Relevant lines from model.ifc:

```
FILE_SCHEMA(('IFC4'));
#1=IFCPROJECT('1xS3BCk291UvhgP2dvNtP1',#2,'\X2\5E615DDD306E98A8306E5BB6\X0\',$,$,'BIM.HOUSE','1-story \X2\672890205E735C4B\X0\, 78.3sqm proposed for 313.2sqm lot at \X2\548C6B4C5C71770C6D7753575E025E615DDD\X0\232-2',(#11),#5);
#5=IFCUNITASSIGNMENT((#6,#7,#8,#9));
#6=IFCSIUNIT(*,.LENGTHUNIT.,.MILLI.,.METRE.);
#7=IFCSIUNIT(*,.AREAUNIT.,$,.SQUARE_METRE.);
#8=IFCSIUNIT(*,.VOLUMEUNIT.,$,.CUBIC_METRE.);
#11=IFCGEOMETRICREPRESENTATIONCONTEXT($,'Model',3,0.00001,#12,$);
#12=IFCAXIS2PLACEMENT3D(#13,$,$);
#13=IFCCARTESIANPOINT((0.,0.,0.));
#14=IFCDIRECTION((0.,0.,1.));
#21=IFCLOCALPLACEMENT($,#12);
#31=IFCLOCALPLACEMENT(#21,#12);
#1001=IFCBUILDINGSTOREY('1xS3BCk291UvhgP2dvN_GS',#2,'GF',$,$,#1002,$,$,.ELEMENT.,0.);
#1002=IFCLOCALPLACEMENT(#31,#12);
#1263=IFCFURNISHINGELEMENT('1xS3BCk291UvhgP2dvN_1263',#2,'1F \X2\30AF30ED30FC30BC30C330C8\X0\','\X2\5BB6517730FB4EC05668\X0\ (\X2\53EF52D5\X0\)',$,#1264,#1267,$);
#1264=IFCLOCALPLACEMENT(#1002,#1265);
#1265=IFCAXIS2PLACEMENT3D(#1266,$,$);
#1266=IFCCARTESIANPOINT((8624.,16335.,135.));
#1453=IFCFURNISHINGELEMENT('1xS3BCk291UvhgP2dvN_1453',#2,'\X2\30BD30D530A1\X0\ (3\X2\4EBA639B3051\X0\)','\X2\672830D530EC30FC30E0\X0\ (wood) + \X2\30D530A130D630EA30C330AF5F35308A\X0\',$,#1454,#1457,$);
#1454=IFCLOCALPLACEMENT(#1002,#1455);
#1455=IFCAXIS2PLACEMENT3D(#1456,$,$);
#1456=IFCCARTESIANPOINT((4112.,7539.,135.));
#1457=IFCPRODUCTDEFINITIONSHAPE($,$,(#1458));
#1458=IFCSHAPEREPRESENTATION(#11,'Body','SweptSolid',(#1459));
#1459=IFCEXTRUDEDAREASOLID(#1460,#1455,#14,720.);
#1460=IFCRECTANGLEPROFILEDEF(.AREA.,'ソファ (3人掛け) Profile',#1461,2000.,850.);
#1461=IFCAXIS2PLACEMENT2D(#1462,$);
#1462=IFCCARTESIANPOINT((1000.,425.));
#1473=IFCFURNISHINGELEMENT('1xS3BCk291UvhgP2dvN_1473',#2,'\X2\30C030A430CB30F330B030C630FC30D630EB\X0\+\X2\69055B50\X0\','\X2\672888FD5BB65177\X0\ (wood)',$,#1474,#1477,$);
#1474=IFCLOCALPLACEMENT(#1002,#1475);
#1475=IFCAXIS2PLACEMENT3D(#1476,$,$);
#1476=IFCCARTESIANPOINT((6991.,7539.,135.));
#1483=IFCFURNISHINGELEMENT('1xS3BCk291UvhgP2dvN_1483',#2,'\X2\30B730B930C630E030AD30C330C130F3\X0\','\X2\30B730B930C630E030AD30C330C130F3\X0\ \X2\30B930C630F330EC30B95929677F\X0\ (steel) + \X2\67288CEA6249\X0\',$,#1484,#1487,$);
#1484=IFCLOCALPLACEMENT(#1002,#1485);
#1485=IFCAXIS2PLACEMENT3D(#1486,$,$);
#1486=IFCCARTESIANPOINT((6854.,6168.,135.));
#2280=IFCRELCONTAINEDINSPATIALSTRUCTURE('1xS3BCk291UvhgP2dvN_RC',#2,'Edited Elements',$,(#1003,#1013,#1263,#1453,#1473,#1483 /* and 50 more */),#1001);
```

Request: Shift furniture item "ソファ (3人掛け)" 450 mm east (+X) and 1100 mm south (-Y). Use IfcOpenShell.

```python
import ifcopenshell
import ifcopenshell.api.geometry
import ifcopenshell.util.placement

model = ifcopenshell.open("model.ifc")

item = model.by_guid("1xS3BCk291UvhgP2dvN_1453")
matrix = ifcopenshell.util.placement.get_local_placement(item.ObjectPlacement)
matrix[0, 3] += 450.0
matrix[1, 3] -= 1100.0
ifcopenshell.api.geometry.edit_object_placement(model, product=item, matrix=matrix, is_si=False)

print(ifcopenshell.util.placement.get_local_placement(item.ObjectPlacement).round(3) + 0.0)

model.write("model_edited.ifc")
```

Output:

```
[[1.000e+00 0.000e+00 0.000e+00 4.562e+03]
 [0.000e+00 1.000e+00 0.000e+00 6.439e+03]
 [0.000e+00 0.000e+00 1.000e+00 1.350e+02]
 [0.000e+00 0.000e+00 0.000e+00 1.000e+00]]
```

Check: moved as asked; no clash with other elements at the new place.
